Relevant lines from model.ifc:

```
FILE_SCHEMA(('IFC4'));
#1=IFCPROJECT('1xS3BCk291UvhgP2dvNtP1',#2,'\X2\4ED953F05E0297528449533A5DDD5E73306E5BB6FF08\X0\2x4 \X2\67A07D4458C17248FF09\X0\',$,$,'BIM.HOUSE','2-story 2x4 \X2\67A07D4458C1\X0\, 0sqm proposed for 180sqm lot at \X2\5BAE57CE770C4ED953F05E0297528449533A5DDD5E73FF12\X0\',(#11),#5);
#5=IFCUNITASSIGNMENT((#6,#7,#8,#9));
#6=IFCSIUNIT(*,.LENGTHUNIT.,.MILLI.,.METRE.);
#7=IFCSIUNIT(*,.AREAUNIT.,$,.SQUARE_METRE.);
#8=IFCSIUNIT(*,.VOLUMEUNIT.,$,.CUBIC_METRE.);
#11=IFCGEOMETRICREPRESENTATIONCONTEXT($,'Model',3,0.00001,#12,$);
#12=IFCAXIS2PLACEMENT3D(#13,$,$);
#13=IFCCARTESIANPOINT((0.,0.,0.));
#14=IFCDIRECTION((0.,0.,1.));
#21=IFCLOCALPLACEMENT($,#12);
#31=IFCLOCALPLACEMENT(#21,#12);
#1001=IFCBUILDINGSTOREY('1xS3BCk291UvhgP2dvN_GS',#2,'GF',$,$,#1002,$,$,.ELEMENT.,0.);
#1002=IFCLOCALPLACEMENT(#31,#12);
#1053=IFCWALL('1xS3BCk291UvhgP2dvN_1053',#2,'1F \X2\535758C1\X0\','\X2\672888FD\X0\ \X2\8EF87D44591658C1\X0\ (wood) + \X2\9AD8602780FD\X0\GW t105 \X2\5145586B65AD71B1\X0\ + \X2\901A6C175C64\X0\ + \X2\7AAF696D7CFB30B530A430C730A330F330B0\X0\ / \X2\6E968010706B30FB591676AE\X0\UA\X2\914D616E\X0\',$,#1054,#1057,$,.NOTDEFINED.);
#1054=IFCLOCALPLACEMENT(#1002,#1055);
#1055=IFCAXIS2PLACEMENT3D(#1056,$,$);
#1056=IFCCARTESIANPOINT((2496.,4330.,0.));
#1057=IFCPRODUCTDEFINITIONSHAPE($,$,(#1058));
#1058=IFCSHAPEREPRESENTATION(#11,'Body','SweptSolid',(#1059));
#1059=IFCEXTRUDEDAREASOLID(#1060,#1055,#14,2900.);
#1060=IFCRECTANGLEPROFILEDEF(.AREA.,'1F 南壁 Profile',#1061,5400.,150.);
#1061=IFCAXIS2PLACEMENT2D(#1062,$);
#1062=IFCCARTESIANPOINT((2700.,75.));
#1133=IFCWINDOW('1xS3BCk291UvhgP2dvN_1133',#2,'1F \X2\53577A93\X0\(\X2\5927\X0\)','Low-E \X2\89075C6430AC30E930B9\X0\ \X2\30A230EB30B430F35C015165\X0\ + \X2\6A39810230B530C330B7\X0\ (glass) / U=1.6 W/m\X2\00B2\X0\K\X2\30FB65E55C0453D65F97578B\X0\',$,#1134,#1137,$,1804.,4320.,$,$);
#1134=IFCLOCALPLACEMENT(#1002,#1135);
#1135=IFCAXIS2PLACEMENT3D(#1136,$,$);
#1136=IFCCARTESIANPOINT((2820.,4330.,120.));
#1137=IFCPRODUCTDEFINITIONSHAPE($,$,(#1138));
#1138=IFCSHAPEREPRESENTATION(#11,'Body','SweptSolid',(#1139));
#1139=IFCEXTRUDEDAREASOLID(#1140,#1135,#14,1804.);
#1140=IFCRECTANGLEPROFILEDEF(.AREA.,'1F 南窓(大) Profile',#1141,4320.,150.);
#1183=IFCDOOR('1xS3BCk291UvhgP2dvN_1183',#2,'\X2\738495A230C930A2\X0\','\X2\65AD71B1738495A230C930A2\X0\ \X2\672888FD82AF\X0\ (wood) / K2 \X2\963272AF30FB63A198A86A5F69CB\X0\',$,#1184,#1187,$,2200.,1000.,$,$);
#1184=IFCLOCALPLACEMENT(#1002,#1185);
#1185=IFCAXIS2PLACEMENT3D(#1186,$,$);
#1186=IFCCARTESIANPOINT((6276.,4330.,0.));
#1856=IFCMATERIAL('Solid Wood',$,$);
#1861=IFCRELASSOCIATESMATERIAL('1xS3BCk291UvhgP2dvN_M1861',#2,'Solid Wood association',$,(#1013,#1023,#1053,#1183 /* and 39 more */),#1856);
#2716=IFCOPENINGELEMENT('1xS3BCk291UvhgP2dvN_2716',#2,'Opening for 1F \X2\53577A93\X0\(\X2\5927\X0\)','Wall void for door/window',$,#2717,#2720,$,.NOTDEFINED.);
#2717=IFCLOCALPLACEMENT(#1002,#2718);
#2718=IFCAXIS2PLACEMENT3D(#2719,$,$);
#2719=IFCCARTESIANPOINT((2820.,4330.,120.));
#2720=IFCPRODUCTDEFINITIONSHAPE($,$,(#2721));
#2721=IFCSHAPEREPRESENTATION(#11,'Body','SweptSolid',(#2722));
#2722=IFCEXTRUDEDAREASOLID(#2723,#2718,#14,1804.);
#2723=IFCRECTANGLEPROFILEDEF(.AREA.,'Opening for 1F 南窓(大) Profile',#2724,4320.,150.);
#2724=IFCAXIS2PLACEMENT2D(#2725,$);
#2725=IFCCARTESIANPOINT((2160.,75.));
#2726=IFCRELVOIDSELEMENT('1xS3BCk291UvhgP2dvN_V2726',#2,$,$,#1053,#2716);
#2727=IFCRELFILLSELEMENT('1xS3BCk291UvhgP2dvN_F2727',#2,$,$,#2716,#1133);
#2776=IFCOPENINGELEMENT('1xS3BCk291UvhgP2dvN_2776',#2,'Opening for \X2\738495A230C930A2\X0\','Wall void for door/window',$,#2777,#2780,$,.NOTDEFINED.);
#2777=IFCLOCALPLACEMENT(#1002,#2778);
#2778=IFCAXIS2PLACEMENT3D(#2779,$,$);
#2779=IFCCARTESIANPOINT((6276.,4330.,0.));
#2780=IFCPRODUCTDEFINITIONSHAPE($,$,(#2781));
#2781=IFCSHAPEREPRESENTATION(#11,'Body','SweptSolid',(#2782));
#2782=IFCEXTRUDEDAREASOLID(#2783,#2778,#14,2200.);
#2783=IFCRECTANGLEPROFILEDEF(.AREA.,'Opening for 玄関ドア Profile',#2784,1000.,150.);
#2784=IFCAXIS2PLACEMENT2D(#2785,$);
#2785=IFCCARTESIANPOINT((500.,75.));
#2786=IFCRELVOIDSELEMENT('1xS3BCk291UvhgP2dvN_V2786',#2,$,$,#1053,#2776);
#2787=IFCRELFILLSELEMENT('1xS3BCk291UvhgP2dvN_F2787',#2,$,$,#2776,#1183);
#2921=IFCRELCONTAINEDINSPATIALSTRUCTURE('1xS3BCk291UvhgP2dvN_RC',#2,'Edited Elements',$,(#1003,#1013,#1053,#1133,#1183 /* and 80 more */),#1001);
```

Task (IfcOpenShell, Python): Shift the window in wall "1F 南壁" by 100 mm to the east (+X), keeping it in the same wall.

```python
import ifcopenshell
import ifcopenshell.api.geometry
import ifcopenshell.util.placement

model = ifcopenshell.open("model.ifc")

window = model.by_guid("1xS3BCk291UvhgP2dvN_1133")
opening = window.FillsVoids[0].RelatingOpeningElement
wall = opening.VoidsElements[0].RelatingBuildingElement

wall_matrix = ifcopenshell.util.placement.get_local_placement(wall.ObjectPlacement)
shift = wall_matrix[:3, 0] * 100.0
before = ifcopenshell.util.placement.get_local_placement(window.ObjectPlacement)[:3, 3].copy()

# The window is not placed relative to its opening, so move both.
for product in (opening, window):
    matrix = ifcopenshell.util.placement.get_local_placement(product.ObjectPlacement)
    matrix[:3, 3] += shift
    ifcopenshell.api.geometry.edit_object_placement(model, product=product, matrix=matrix, is_si=False)

after = ifcopenshell.util.placement.get_local_placement(window.ObjectPlacement)[:3, 3]
print("window moved by", (after - before).round(3) + 0.0)

model.write("model_v2.ifc")
```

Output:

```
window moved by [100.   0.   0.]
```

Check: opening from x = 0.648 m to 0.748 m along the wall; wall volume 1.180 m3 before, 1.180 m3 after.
